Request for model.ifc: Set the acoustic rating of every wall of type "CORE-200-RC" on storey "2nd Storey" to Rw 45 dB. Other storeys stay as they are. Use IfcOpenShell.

First a look at what the model holds.

```python
import ifcopenshell
import ifcopenshell.util.element

model = ifcopenshell.open("model.ifc")
print(model.schema)
storey = next(s for s in model.by_type("IfcBuildingStorey") if s.Name == "2nd Storey")
walls = [e for e in ifcopenshell.util.element.get_decomposition(storey) if e.is_a("IfcWall")]
seen = {}
for e in walls:
    element_type = ifcopenshell.util.element.get_type(e)
    key = (element_type.Name if element_type != e and element_type else None, ifcopenshell.util.element.get_pset(e, "Pset_WallCommon", "AcousticRating"))
    seen[key] = seen.get(key, 0) + 1
for (name, value), count in sorted(seen.items(), key=str):
    print(count, "x", name, "|", value)
```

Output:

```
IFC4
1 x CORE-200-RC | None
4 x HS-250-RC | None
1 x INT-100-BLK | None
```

```python
import ifcopenshell
import ifcopenshell.api.pset
import ifcopenshell.util.element

model = ifcopenshell.open("model.ifc")

storey = next(s for s in model.by_type("IfcBuildingStorey") if s.Name == "2nd Storey")
walls = [e for e in ifcopenshell.util.element.get_decomposition(storey) if e.is_a("IfcWall")]

count = 0
for e in walls:
    element_type = ifcopenshell.util.element.get_type(e)
    if element_type in (None, e) or element_type.Name != "CORE-200-RC":
        continue
    # add_pset returns the element's existing set when there is one.
    pset = ifcopenshell.api.pset.add_pset(model, product=e, name="Pset_WallCommon")
    ifcopenshell.api.pset.edit_pset(model, pset=pset, properties={"AcousticRating": "Rw 45 dB"})
    count += 1

print(count, "walls updated")

model.write("model_updated.ifc")
```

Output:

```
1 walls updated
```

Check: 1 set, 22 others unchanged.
